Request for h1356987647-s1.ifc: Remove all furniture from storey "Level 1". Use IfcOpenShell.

First a look at what the model holds.

```python
import ifcopenshell
import ifcopenshell.util.element

model = ifcopenshell.open("h1356987647-s1.ifc")
print(model.schema)
storey = next(s for s in model.by_type("IfcBuildingStorey") if s.Name == "Level 1")
furniture = [e for e in ifcopenshell.util.element.get_decomposition(storey) if e.is_a("IfcFurnishingElement")]
seen = {}
for e in furniture:
    element_type = ifcopenshell.util.element.get_type(e)
    name = element_type.Name if element_type not in (None, e) else None
    seen[name] = seen.get(name, 0) + 1
for name, count in sorted(seen.items(), key=str):
    print(count, "x", name)
```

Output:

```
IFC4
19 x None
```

```python
import ifcopenshell
import ifcopenshell.api.root
import ifcopenshell.util.element

model = ifcopenshell.open("h1356987647-s1.ifc")

storey = next(s for s in model.by_type("IfcBuildingStorey") if s.Name == "Level 1")
furniture = [e for e in ifcopenshell.util.element.get_decomposition(storey) if e.is_a("IfcFurnishingElement")]

for e in furniture:
    ifcopenshell.api.root.remove_product(model, product=e)
print(len(furniture), "removed")

model.write("h1356987647-s1_updated.ifc")
```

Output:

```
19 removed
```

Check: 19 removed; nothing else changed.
